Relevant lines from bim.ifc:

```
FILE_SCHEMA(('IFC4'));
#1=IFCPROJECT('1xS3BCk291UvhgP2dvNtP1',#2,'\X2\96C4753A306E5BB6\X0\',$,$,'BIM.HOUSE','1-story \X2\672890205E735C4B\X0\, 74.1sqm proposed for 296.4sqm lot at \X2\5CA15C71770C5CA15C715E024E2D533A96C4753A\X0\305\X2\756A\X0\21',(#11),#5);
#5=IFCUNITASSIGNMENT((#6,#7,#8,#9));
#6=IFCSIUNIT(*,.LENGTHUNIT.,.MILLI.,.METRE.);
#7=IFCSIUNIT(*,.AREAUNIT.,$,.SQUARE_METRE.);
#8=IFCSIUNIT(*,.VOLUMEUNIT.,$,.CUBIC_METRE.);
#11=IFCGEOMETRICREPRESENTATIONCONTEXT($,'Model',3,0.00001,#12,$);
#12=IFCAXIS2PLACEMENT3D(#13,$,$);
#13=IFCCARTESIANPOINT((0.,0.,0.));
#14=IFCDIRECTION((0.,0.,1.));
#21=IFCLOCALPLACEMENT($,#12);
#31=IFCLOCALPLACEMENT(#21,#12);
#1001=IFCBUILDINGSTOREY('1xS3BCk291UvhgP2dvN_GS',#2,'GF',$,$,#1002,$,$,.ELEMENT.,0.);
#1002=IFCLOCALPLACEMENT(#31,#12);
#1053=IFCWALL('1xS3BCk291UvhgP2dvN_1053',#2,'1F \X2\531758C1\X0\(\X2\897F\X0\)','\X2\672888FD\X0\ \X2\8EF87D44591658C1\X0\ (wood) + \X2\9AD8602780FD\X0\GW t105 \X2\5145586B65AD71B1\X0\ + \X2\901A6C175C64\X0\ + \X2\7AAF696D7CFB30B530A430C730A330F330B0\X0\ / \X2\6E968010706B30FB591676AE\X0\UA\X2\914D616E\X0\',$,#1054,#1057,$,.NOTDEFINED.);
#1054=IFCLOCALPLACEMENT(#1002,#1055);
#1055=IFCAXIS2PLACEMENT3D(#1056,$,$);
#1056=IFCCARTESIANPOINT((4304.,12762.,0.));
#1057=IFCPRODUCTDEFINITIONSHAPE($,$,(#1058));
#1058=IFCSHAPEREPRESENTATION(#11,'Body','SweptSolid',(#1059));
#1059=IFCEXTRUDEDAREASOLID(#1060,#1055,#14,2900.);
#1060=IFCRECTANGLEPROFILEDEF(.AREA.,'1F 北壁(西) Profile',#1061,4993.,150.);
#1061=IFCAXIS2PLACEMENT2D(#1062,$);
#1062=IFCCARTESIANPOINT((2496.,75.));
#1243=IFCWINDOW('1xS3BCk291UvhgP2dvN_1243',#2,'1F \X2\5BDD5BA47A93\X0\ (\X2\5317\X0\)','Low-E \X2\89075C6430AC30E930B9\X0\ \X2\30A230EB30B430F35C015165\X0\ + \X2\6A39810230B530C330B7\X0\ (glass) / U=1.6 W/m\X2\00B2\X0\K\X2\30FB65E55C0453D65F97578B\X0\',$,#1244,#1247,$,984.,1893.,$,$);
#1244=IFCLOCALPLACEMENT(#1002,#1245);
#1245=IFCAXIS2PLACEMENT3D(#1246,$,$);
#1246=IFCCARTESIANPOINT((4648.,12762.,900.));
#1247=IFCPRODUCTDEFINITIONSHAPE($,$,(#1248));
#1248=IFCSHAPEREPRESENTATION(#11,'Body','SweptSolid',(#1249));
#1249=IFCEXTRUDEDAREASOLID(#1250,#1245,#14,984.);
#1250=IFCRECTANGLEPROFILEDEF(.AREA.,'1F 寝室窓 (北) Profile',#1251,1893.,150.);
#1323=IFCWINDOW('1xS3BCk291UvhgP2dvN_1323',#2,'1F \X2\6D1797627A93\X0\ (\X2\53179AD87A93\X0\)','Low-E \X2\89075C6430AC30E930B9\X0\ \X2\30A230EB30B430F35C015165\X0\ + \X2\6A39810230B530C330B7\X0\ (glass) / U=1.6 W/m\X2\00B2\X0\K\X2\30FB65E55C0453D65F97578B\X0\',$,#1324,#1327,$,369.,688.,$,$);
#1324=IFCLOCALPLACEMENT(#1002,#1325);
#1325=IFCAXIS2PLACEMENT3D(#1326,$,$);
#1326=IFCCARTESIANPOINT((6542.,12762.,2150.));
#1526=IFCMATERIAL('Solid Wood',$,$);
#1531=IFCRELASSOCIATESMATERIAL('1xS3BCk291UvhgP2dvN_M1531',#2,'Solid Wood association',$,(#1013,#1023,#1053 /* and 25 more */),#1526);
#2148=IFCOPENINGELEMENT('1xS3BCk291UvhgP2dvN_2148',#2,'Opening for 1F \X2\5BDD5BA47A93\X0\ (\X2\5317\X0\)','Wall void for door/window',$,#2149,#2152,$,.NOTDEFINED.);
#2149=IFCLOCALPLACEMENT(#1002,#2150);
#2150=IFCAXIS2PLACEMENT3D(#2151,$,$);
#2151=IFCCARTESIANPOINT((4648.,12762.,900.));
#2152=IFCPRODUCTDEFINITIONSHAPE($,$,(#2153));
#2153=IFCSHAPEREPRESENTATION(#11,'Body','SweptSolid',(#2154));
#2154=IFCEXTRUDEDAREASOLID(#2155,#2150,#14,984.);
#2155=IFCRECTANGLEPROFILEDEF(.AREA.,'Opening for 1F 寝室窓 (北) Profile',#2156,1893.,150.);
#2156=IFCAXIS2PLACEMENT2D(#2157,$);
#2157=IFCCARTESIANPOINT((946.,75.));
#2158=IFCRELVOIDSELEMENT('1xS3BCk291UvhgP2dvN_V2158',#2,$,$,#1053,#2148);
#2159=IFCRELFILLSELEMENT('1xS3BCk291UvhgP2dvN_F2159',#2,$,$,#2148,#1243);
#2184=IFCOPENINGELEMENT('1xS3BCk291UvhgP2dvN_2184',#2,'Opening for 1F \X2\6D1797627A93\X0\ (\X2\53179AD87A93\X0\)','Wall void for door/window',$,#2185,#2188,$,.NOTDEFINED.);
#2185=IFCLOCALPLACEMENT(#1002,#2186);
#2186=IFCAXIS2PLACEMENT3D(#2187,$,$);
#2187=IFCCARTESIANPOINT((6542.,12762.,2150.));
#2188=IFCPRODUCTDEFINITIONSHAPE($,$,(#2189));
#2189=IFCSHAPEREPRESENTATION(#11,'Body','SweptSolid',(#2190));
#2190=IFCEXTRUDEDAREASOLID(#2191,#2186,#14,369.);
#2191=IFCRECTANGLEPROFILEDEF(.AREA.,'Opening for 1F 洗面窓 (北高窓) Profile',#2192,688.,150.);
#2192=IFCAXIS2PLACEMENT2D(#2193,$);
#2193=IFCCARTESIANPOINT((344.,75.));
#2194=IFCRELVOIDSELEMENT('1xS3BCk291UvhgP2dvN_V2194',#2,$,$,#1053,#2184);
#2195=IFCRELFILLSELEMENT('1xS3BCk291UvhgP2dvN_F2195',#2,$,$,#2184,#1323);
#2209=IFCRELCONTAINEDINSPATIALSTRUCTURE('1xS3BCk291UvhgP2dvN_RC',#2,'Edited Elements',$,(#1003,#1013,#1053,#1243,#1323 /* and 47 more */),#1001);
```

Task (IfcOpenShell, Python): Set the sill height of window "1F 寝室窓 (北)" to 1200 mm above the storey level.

```python
import numpy as np
import ifcopenshell
import ifcopenshell.api.geometry
import ifcopenshell.geom
import ifcopenshell.util.element
import ifcopenshell.util.placement
import ifcopenshell.util.shape
import ifcopenshell.util.unit

model = ifcopenshell.open("bim.ifc")
unit_scale = ifcopenshell.util.unit.calculate_unit_scale(model)

window = model.by_id(1243)
opening = window.FillsVoids[0].RelatingOpeningElement
storey = ifcopenshell.util.element.get_container(window, ifc_class="IfcBuildingStorey")
level = ifcopenshell.util.placement.get_local_placement(storey.ObjectPlacement)[2, 3]

# The opening's origin need not be at the sill, so measure its lowest point.
shape = ifcopenshell.geom.create_shape(ifcopenshell.geom.settings(), opening)
bottom = ifcopenshell.util.shape.get_shape_bottom_elevation(shape, shape.geometry) / unit_scale
dz = level + 1.2 / unit_scale - bottom

shift = np.array([0.0, 0.0, dz])
# The window is not placed relative to its opening, so move both.
for product in (opening, window):
    matrix = ifcopenshell.util.placement.get_local_placement(product.ObjectPlacement)
    matrix[:3, 3] += shift
    ifcopenshell.api.geometry.edit_object_placement(model, product=product, matrix=matrix, is_si=False)

print(f"moved by {dz * unit_scale:+.3f} m")

model.write("bim_v2.ifc")
```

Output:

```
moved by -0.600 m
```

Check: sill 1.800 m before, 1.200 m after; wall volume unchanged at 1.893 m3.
